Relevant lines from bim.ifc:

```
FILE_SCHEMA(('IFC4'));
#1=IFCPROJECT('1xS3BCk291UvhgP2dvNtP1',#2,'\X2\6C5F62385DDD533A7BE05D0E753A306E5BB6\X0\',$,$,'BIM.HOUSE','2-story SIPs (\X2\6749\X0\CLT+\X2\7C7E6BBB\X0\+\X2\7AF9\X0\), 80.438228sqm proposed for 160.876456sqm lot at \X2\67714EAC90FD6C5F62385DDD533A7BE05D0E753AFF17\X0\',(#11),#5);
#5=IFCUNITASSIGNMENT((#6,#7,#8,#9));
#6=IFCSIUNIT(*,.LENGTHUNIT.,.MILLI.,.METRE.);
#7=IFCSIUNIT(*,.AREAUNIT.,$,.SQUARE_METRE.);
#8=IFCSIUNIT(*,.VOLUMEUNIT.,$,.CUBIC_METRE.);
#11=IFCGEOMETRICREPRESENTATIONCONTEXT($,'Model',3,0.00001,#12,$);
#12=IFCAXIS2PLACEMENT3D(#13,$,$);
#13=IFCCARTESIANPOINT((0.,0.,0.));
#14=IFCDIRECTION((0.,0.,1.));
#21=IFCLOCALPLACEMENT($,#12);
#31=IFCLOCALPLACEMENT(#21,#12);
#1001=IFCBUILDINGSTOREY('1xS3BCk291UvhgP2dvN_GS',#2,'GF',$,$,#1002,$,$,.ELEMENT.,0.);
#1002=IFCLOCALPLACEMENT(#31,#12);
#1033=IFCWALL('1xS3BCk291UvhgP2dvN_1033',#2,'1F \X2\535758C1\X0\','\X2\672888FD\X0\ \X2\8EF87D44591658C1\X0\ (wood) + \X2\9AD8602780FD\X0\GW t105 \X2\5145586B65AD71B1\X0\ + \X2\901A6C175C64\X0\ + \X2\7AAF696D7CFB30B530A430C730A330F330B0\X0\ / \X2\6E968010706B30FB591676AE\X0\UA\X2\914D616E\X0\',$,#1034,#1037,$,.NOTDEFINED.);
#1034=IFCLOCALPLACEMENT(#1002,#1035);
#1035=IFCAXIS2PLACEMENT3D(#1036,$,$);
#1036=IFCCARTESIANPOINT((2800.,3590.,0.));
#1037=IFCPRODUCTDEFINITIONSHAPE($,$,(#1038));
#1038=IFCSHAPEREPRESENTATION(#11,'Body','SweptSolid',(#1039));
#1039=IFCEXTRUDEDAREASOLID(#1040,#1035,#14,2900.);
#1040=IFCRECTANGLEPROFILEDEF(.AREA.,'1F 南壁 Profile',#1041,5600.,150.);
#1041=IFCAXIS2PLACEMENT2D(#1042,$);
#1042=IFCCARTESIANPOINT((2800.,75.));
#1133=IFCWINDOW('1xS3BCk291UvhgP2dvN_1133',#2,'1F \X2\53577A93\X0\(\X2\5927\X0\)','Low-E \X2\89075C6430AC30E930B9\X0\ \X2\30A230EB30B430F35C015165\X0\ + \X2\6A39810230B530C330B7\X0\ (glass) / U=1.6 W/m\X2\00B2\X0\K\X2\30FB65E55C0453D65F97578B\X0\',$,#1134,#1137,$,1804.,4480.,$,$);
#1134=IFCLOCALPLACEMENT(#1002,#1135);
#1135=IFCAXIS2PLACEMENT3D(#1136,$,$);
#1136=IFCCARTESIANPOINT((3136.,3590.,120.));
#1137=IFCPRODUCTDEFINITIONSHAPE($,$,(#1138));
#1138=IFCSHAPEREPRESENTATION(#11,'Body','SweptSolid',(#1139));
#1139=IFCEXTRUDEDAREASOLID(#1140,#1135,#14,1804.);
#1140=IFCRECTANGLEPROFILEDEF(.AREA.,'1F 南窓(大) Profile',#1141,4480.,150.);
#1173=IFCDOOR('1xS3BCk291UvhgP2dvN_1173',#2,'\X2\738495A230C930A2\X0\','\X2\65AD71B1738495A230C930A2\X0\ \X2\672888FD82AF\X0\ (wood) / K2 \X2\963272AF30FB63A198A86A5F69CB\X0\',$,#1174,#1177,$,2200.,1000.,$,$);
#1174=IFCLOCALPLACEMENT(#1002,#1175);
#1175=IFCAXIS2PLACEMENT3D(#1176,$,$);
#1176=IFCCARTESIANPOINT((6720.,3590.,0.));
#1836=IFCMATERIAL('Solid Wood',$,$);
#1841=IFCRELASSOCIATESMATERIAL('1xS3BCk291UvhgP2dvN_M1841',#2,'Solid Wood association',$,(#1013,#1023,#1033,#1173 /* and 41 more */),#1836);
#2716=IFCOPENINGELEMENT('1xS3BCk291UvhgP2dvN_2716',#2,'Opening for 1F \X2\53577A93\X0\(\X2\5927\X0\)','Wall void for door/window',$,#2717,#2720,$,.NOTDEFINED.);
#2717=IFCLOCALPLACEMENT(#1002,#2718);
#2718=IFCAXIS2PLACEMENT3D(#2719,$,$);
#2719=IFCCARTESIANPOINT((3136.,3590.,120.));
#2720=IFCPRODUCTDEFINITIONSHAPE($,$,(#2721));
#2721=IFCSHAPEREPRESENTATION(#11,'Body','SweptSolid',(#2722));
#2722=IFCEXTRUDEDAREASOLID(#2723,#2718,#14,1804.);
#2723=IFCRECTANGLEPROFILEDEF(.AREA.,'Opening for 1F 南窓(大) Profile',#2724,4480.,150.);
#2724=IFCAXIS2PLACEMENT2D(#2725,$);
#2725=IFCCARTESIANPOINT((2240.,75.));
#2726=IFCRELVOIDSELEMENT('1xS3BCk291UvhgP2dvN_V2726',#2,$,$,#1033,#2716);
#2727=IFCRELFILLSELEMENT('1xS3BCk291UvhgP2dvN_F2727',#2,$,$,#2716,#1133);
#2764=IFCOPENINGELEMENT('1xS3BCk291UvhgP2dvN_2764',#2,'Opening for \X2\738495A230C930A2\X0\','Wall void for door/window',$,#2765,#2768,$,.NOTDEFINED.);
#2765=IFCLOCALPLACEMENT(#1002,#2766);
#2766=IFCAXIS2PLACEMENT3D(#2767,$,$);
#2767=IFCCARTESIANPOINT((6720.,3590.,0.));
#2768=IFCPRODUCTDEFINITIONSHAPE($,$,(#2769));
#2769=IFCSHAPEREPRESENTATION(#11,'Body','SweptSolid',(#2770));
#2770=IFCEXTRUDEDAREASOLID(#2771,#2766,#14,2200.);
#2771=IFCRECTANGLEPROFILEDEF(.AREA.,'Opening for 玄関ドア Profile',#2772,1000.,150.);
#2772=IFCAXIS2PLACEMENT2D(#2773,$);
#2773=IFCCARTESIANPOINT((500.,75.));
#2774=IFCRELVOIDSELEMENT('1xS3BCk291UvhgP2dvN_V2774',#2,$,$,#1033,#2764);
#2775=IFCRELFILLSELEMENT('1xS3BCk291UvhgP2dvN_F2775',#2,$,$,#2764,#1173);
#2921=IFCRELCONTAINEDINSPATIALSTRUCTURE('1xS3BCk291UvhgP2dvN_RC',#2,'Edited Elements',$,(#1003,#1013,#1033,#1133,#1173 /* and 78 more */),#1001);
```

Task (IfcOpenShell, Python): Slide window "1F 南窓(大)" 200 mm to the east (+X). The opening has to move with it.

```python
import ifcopenshell
import ifcopenshell.api.geometry
import ifcopenshell.util.placement
import ifcopenshell.util.unit

model = ifcopenshell.open("bim.ifc")
unit_scale = ifcopenshell.util.unit.calculate_unit_scale(model)

window = model.by_id(1133)
opening = window.FillsVoids[0].RelatingOpeningElement
wall = opening.VoidsElements[0].RelatingBuildingElement

wall_matrix = ifcopenshell.util.placement.get_local_placement(wall.ObjectPlacement)
shift = wall_matrix[:3, 0] * 0.2 / unit_scale
before = ifcopenshell.util.placement.get_local_placement(window.ObjectPlacement)[:3, 3].copy()

# The window is not placed relative to its opening, so move both.
for product in (opening, window):
    matrix = ifcopenshell.util.placement.get_local_placement(product.ObjectPlacement)
    matrix[:3, 3] += shift
    ifcopenshell.api.geometry.edit_object_placement(model, product=product, matrix=matrix, is_si=False)

after = ifcopenshell.util.placement.get_local_placement(window.ObjectPlacement)[:3, 3]
print("window moved by", (after - before).round(3) + 0.0)

model.write("bim_updated.ifc")
```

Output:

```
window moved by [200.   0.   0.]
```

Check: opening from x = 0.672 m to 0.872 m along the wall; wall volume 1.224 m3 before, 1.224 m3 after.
